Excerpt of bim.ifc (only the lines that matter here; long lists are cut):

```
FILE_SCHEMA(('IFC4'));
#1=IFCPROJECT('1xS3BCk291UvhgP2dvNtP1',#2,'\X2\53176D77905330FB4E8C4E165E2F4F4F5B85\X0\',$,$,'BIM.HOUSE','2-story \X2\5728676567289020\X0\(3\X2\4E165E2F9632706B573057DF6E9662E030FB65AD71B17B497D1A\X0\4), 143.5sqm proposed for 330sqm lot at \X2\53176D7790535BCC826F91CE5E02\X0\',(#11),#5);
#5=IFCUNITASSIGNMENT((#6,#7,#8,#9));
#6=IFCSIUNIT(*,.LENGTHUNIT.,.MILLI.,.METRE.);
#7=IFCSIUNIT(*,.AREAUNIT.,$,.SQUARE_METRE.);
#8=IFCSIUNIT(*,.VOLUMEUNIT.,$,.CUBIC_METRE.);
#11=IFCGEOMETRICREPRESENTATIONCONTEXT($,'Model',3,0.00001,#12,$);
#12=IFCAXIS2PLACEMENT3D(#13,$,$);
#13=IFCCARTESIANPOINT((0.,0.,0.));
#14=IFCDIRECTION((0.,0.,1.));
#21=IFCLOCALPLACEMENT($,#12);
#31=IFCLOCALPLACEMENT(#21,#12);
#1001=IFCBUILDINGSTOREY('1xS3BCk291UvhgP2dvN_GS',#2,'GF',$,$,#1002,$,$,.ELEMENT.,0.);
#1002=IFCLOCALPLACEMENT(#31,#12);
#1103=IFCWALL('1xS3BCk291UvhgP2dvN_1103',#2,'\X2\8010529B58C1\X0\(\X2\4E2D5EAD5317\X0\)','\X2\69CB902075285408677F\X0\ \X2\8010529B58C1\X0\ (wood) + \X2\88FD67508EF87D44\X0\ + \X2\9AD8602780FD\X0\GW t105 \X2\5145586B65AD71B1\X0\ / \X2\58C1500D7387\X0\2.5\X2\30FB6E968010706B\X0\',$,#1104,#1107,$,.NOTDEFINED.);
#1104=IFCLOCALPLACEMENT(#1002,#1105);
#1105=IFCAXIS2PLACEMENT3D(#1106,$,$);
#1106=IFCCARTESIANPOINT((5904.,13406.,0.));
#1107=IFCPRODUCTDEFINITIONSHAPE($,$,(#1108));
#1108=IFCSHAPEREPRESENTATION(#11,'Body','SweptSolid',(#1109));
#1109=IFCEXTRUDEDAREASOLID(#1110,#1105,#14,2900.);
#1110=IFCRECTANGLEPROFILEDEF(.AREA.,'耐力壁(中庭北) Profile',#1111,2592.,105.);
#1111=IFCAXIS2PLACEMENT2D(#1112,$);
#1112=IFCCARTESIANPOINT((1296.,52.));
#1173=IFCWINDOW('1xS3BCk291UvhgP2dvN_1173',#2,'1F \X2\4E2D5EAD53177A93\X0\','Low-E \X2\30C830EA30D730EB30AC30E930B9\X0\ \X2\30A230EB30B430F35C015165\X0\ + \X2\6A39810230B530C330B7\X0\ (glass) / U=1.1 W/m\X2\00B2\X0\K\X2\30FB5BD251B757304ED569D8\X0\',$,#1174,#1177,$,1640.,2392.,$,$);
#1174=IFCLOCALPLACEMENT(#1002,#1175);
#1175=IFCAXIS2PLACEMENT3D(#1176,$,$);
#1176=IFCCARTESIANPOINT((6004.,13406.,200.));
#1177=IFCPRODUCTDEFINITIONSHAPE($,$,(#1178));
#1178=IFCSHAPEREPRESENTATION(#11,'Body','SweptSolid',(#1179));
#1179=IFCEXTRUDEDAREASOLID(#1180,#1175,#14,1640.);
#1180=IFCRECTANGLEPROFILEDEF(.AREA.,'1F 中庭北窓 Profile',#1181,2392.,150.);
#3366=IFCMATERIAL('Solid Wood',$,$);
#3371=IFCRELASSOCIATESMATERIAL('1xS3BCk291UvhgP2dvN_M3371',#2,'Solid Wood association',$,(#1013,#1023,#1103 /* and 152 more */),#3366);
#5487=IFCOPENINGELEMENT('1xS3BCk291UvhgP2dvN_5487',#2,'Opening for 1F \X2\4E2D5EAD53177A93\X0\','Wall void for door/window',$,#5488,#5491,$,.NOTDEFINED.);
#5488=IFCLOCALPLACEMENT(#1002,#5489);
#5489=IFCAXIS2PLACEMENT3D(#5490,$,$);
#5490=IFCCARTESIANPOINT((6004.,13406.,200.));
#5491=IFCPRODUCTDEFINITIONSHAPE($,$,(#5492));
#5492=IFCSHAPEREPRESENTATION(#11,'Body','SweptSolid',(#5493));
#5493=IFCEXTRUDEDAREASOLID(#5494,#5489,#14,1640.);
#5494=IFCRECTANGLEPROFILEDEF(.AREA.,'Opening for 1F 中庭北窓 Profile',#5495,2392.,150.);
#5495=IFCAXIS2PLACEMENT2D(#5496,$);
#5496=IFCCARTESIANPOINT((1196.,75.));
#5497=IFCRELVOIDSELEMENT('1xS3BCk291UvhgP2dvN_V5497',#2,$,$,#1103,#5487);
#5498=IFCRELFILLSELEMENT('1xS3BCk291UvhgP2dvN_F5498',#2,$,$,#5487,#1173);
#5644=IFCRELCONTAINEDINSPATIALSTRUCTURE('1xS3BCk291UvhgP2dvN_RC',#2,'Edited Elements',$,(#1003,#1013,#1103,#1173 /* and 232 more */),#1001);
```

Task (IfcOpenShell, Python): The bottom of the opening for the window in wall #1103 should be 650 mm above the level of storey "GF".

```python
import numpy as np
import ifcopenshell
import ifcopenshell.api.geometry
import ifcopenshell.geom
import ifcopenshell.util.element
import ifcopenshell.util.placement
import ifcopenshell.util.shape
import ifcopenshell.util.unit

model = ifcopenshell.open("bim.ifc")
unit_scale = ifcopenshell.util.unit.calculate_unit_scale(model)

window = model.by_guid("1xS3BCk291UvhgP2dvN_1173")
opening = window.FillsVoids[0].RelatingOpeningElement
storey = ifcopenshell.util.element.get_container(window, ifc_class="IfcBuildingStorey")
level = ifcopenshell.util.placement.get_local_placement(storey.ObjectPlacement)[2, 3]

# The opening's origin need not be at the sill, so measure its lowest point.
shape = ifcopenshell.geom.create_shape(ifcopenshell.geom.settings(), opening)
bottom = ifcopenshell.util.shape.get_shape_bottom_elevation(shape, shape.geometry) / unit_scale
dz = level + 650.0 - bottom

shift = np.array([0.0, 0.0, dz])
# The window is not placed relative to its opening, so move both.
for product in (opening, window):
    matrix = ifcopenshell.util.placement.get_local_placement(product.ObjectPlacement)
    matrix[:3, 3] += shift
    ifcopenshell.api.geometry.edit_object_placement(model, product=product, matrix=matrix, is_si=False)

print(f"moved by {dz * unit_scale:+.3f} m")

model.write("bim_rev.ifc")
```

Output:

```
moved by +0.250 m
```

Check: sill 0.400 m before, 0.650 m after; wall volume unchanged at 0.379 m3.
